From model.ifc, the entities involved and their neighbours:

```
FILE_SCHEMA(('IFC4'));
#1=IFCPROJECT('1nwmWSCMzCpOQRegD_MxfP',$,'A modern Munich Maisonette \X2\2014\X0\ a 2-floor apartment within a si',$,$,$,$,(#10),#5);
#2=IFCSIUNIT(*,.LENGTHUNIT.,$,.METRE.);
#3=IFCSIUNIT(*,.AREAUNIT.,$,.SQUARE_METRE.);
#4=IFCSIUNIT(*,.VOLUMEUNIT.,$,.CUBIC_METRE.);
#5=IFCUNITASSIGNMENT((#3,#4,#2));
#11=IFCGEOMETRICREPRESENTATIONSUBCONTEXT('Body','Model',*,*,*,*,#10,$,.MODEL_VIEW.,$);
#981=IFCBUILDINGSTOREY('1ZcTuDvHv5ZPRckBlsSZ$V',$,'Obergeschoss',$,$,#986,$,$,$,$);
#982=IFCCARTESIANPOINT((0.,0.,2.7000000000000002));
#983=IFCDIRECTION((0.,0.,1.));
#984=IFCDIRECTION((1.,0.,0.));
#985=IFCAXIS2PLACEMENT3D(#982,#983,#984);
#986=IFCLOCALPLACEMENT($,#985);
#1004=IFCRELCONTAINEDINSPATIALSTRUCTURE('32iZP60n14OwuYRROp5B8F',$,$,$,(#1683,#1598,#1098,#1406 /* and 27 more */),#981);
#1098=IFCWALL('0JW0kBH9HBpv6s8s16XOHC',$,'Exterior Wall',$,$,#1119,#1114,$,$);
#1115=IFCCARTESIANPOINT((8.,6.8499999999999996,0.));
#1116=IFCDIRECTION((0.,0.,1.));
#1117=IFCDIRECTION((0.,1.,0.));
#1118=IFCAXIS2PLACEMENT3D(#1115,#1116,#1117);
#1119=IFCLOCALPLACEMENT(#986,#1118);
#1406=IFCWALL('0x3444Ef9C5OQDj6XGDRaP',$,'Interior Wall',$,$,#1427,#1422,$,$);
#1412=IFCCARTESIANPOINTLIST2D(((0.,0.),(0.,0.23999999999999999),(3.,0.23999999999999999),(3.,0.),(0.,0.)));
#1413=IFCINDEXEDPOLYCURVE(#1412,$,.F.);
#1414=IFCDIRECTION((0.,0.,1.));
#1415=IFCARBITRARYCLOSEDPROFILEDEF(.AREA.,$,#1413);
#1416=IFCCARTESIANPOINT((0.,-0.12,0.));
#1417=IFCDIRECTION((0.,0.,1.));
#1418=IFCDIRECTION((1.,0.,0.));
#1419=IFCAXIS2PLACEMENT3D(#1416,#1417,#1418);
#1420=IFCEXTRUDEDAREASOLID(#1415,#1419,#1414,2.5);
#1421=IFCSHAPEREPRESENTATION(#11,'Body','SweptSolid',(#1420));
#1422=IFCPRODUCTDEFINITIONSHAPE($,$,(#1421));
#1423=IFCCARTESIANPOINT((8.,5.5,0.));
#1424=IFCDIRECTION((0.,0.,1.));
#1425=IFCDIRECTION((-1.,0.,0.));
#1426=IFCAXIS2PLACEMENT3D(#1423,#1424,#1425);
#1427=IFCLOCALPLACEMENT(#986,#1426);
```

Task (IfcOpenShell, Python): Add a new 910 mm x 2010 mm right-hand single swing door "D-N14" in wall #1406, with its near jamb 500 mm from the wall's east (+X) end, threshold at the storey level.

```python
import numpy as np
import ifcopenshell
import ifcopenshell.api.feature
import ifcopenshell.api.geometry
import ifcopenshell.api.root
import ifcopenshell.api.spatial
import ifcopenshell.geom
import ifcopenshell.util.element
import ifcopenshell.util.placement
import ifcopenshell.util.representation
import ifcopenshell.util.shape
import ifcopenshell.util.unit

model = ifcopenshell.open("model.ifc")
unit_scale = ifcopenshell.util.unit.calculate_unit_scale(model)
settings = ifcopenshell.geom.settings()


def volume(element):
    """Net volume in cubic metres, openings subtracted."""
    shape = ifcopenshell.geom.create_shape(settings, element)
    return ifcopenshell.util.shape.get_volume(shape.geometry)


wall = model.by_guid("0x3444Ef9C5OQDj6XGDRaP")
storey = ifcopenshell.util.element.get_container(wall, ifc_class="IfcBuildingStorey")
context = ifcopenshell.util.representation.get_context(model, "Model", "Body", "MODEL_VIEW")
before = volume(wall)

width, height, from_end, sill = 0.91, 2.01, 0.5, 0.0  # metres

# The wall runs along its own X axis, and the end named is its -X end.
wall_shape = ifcopenshell.geom.create_shape(settings, wall)
x, y, z = ifcopenshell.util.shape.get_vertices(wall_shape.geometry).T
start = x.min() + from_end
face, thickness = float(y.min()), float(y.max() - y.min())
wall_matrix = ifcopenshell.util.placement.get_local_placement(wall.ObjectPlacement)
level = ifcopenshell.util.placement.get_local_placement(storey.ObjectPlacement)[2, 3]


def in_wall(x, y):
    """Placement at x, y metres in the wall's axes, at sill height."""
    matrix = wall_matrix.copy()
    matrix[:, 3] = wall_matrix @ np.array([x / unit_scale, y / unit_scale, 0.0, 1.0])
    matrix[2, 3] = level + sill / unit_scale
    return matrix


# Opening: a box that overshoots both wall faces by 50 mm.
opening = ifcopenshell.api.root.create_entity(model, ifc_class="IfcOpeningElement", predefined_type="OPENING")
box = ifcopenshell.api.geometry.add_wall_representation(
    model, context=context, length=width, height=height, thickness=thickness + 0.1
)
ifcopenshell.api.geometry.assign_representation(model, product=opening, representation=box)
ifcopenshell.api.geometry.edit_object_placement(model, product=opening, matrix=in_wall(start, face - 0.05), is_si=False)
ifcopenshell.api.feature.add_feature(model, feature=opening, element=wall)

door = ifcopenshell.api.root.create_entity(model, ifc_class="IfcDoor", name="D-N14", predefined_type="DOOR")
door.OverallWidth, door.OverallHeight = width / unit_scale, height / unit_scale
door.OperationType = "SINGLE_SWING_RIGHT"
body = ifcopenshell.api.geometry.add_door_representation(
    model,
    context=context,
    overall_width=door.OverallWidth,
    overall_height=door.OverallHeight,
    operation_type="SINGLE_SWING_RIGHT",
    lining_properties={"LiningDepth": thickness / unit_scale, "ThresholdDepth": thickness / unit_scale},
)
ifcopenshell.api.geometry.assign_representation(model, product=door, representation=body)
ifcopenshell.api.spatial.assign_container(model, products=[door], relating_structure=storey)
ifcopenshell.api.feature.add_filling(model, opening=opening, element=door)

# The lining spans the wall, so the door starts at the wall face.
ifcopenshell.api.geometry.edit_object_placement(model, product=door, matrix=in_wall(start, face), is_si=False)

after = volume(wall)

print(f"wall volume {before:.3f} -> {after:.3f} m3")

model.write("model_v2.ifc")
```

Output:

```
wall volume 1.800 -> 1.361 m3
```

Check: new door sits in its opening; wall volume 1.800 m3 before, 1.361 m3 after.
